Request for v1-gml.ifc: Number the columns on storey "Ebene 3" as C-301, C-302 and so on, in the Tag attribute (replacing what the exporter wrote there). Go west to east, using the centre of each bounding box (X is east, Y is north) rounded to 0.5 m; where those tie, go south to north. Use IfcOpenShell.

First a look at what the model holds.

```python
import ifcopenshell
import ifcopenshell.util.element
import ifcopenshell.util.placement

model = ifcopenshell.open("v1-gml.ifc")
print(model.schema)
storey = next(s for s in model.by_type("IfcBuildingStorey") if s.Name == "Ebene 3")
columns = [e for e in ifcopenshell.util.element.get_decomposition(storey) if e.is_a("IfcColumn")]
for e in sorted(columns, key=lambda e: e.id()):
    origin = ifcopenshell.util.placement.get_local_placement(e.ObjectPlacement)[:3, 3]
    print(e.id(), e.Tag, e.Name, origin.round(2) + 0.0, sep=" | ")
```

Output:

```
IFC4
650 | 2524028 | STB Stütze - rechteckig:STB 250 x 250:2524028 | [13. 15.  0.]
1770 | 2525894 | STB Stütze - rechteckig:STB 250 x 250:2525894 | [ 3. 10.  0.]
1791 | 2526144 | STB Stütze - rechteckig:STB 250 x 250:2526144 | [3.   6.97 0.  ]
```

```python
import ifcopenshell
import ifcopenshell.geom
import ifcopenshell.util.element
import ifcopenshell.util.shape

model = ifcopenshell.open("v1-gml.ifc")
settings = ifcopenshell.geom.settings()
settings.set("use-world-coords", True)


def centre(element):
    shape = ifcopenshell.geom.create_shape(settings, element)
    return ifcopenshell.util.shape.get_bbox_centroid(shape.geometry)


storey = next(s for s in model.by_type("IfcBuildingStorey") if s.Name == "Ebene 3")
columns = [e for e in ifcopenshell.util.element.get_decomposition(storey) if e.is_a("IfcColumn")]

# Insertion points can sit at a corner or the storey origin, so sort by the geometry (in metres).
centres = {e: centre(e) for e in columns}
columns.sort(key=lambda e: (round(centres[e][0] / 0.5), centres[e][1]))

for i, e in enumerate(columns, start=1):
    number = f"C-3{i:02d}"
    e.Tag = number
    print(e.id(), number)

model.write("v1-gml_edited.ifc")
```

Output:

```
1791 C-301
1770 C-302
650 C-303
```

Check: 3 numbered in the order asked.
